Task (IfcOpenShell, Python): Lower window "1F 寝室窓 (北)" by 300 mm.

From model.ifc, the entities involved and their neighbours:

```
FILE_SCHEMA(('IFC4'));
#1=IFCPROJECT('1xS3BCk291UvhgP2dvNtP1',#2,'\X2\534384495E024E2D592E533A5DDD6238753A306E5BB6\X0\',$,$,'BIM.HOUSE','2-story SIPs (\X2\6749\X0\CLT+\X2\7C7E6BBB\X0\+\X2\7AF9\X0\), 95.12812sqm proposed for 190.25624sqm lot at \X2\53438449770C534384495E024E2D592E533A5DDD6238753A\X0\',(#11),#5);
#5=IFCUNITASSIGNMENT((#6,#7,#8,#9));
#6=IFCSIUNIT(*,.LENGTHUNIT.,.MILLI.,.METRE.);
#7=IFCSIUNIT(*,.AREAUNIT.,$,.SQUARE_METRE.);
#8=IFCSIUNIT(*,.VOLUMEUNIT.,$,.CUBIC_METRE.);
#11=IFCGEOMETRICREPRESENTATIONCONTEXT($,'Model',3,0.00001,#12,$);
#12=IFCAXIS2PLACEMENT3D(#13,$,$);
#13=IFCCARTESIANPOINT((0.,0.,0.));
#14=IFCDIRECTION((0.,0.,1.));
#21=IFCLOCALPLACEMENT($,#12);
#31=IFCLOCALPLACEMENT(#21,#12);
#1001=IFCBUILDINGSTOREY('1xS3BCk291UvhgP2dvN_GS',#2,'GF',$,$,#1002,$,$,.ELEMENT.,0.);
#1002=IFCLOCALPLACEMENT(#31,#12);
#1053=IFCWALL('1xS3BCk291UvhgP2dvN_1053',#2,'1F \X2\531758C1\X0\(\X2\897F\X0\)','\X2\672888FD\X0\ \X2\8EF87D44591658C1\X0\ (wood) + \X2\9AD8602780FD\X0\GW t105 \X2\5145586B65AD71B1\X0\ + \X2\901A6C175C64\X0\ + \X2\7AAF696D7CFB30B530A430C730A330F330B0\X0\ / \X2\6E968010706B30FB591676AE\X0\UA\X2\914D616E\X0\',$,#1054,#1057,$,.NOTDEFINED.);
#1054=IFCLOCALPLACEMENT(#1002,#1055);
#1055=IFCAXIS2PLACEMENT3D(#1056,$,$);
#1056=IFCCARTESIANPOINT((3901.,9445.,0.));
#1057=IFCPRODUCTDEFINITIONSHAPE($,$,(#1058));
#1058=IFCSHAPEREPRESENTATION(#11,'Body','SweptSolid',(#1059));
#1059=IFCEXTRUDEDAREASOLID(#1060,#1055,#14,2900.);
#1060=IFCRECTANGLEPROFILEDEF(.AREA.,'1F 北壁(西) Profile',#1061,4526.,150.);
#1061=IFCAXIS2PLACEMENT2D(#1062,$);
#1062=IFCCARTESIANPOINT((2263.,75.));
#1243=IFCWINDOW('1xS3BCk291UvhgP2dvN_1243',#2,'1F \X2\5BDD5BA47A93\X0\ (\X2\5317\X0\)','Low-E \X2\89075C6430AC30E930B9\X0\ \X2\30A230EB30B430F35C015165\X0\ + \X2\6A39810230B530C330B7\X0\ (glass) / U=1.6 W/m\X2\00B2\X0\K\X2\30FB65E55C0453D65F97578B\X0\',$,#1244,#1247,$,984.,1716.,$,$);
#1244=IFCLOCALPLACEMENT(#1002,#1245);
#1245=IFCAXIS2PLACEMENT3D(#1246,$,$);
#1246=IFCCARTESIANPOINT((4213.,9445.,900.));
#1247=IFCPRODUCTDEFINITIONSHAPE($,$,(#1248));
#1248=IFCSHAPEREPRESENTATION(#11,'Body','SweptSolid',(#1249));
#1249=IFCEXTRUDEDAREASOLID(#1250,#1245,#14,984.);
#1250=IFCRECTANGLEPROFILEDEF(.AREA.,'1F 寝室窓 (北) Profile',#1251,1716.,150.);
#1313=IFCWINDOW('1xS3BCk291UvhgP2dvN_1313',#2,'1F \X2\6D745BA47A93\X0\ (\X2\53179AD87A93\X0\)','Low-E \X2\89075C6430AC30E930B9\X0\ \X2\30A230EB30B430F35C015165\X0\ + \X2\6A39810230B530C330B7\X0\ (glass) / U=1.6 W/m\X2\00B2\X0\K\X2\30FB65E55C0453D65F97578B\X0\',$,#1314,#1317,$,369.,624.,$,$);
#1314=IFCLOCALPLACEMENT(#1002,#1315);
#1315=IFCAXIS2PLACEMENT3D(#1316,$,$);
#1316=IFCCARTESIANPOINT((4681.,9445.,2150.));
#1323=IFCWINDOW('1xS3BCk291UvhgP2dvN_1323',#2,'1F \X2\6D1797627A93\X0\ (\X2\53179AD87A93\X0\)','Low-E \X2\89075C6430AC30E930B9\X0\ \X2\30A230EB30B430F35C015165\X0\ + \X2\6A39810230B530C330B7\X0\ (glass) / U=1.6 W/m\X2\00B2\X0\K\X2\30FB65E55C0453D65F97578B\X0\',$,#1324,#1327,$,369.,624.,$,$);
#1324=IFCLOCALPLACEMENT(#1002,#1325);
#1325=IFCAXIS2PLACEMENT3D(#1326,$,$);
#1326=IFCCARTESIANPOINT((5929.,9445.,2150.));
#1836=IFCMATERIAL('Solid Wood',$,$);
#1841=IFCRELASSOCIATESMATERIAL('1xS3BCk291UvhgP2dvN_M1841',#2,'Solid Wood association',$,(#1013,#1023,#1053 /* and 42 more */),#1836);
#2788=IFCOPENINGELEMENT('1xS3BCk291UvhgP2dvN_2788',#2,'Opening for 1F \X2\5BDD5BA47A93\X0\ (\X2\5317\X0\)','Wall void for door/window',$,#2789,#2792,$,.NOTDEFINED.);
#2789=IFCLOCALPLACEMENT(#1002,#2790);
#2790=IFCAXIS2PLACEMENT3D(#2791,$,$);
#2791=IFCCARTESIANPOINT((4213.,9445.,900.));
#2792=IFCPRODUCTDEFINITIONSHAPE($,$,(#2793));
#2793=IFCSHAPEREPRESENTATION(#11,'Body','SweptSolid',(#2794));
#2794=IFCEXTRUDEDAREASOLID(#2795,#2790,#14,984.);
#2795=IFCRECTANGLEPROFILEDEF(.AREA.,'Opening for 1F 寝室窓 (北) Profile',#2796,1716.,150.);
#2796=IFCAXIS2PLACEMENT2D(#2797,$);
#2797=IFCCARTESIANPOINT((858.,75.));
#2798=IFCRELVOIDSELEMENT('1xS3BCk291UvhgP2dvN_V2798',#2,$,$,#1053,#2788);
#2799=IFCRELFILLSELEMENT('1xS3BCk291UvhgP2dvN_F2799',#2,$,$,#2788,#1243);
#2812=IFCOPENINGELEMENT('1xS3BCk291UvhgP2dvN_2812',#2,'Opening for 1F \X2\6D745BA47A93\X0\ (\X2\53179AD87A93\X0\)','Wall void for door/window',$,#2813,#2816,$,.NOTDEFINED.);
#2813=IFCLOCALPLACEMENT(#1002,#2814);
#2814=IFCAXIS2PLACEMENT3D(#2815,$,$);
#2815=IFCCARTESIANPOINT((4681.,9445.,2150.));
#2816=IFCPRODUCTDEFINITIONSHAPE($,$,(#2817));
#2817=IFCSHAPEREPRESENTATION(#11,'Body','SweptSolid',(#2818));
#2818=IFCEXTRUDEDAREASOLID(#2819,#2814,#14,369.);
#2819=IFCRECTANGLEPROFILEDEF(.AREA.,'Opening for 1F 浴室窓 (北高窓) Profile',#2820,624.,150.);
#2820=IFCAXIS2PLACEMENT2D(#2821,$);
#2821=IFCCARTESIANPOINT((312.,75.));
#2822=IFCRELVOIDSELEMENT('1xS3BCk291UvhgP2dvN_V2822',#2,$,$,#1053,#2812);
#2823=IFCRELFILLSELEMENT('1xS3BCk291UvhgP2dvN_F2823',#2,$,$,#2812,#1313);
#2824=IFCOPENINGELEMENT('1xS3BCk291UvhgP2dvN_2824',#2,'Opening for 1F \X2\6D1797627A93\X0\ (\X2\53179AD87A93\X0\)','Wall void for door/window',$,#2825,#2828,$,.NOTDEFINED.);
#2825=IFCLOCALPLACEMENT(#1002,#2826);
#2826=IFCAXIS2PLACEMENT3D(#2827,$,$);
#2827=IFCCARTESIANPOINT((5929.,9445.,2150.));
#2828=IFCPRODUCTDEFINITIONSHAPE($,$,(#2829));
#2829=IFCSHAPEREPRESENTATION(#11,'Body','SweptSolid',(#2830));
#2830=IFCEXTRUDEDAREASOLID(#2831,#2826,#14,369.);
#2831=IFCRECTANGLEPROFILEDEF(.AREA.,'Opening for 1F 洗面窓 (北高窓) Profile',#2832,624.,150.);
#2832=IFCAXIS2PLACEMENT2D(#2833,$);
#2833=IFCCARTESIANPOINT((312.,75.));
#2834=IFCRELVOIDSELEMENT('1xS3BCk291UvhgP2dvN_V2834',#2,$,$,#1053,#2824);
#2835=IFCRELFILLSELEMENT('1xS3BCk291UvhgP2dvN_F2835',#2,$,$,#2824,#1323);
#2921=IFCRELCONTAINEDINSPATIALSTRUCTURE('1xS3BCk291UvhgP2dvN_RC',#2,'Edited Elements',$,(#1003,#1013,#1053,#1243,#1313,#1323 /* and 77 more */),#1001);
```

```python
import numpy as np
import ifcopenshell
import ifcopenshell.api.geometry
import ifcopenshell.util.placement
import ifcopenshell.util.unit

model = ifcopenshell.open("model.ifc")
unit_scale = ifcopenshell.util.unit.calculate_unit_scale(model)

window = model.by_id(1243)
opening = window.FillsVoids[0].RelatingOpeningElement
dz = -0.3 / unit_scale

shift = np.array([0.0, 0.0, dz])
# The window is not placed relative to its opening, so move both.
for product in (opening, window):
    matrix = ifcopenshell.util.placement.get_local_placement(product.ObjectPlacement)
    matrix[:3, 3] += shift
    ifcopenshell.api.geometry.edit_object_placement(model, product=product, matrix=matrix, is_si=False)

print(f"moved by {dz * unit_scale:+.3f} m")

model.write("model-out.ifc")
```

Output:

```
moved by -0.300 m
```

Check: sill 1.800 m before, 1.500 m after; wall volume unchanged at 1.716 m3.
